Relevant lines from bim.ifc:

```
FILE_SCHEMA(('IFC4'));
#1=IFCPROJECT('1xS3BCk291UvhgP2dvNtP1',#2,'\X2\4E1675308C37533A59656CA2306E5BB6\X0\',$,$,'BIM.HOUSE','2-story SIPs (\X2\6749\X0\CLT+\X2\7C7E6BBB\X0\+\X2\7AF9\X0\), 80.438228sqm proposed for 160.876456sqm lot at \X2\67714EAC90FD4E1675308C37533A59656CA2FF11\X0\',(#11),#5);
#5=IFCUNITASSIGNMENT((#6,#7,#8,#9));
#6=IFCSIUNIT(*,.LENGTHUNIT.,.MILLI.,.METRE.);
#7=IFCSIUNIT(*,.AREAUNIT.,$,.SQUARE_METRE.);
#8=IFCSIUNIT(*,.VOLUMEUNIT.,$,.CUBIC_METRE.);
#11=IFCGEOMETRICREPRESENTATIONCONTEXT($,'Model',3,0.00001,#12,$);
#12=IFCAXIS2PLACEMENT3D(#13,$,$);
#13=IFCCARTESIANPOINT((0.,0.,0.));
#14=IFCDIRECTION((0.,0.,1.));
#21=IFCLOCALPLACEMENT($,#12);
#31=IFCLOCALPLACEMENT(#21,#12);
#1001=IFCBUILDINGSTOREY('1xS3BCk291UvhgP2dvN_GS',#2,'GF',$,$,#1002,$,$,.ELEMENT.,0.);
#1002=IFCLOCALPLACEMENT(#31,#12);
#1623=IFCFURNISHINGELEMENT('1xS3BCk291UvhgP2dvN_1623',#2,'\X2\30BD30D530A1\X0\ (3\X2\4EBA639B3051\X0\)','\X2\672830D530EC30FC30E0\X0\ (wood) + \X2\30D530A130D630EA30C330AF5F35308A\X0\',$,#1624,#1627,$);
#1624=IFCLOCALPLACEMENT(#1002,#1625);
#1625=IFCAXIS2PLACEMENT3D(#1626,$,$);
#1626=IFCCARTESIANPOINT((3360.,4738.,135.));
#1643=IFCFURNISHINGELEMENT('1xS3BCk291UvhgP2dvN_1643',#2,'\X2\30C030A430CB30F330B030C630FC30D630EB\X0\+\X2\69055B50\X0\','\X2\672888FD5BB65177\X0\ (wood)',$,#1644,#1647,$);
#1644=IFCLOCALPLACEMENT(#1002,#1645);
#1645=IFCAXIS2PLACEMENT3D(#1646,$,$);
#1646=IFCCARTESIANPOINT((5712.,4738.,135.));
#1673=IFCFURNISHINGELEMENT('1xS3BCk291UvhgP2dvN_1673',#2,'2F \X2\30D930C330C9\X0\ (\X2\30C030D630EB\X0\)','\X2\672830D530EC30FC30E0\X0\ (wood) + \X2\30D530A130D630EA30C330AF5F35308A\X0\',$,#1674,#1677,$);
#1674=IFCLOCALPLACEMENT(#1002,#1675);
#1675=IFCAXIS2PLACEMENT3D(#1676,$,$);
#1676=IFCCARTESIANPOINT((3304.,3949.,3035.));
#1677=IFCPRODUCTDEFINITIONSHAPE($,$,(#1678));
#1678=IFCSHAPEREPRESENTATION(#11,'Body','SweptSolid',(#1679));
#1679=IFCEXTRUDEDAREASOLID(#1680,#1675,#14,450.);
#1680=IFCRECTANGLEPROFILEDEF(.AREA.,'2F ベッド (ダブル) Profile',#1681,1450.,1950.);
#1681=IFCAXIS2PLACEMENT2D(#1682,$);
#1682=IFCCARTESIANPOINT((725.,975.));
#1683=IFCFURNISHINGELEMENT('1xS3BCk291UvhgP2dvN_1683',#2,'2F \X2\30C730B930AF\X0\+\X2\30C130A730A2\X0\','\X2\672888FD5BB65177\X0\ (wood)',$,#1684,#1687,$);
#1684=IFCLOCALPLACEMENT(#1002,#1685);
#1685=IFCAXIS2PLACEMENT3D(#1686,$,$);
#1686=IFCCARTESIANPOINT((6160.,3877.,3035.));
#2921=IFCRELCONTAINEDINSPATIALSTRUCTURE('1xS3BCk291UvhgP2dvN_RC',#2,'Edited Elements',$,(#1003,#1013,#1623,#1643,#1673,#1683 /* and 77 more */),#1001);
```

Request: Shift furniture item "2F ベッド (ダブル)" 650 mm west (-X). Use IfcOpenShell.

```python
import ifcopenshell
import ifcopenshell.api.geometry
import ifcopenshell.util.placement

model = ifcopenshell.open("bim.ifc")

item = model.by_guid("1xS3BCk291UvhgP2dvN_1673")
matrix = ifcopenshell.util.placement.get_local_placement(item.ObjectPlacement)
matrix[0, 3] -= 650.0
ifcopenshell.api.geometry.edit_object_placement(model, product=item, matrix=matrix, is_si=False)

print(ifcopenshell.util.placement.get_local_placement(item.ObjectPlacement).round(3) + 0.0)

model.write("bim_v2.ifc")
```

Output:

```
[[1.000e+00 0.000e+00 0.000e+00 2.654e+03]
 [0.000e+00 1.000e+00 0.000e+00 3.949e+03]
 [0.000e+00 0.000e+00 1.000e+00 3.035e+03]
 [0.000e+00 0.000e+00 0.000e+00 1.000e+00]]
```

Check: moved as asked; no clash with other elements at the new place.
